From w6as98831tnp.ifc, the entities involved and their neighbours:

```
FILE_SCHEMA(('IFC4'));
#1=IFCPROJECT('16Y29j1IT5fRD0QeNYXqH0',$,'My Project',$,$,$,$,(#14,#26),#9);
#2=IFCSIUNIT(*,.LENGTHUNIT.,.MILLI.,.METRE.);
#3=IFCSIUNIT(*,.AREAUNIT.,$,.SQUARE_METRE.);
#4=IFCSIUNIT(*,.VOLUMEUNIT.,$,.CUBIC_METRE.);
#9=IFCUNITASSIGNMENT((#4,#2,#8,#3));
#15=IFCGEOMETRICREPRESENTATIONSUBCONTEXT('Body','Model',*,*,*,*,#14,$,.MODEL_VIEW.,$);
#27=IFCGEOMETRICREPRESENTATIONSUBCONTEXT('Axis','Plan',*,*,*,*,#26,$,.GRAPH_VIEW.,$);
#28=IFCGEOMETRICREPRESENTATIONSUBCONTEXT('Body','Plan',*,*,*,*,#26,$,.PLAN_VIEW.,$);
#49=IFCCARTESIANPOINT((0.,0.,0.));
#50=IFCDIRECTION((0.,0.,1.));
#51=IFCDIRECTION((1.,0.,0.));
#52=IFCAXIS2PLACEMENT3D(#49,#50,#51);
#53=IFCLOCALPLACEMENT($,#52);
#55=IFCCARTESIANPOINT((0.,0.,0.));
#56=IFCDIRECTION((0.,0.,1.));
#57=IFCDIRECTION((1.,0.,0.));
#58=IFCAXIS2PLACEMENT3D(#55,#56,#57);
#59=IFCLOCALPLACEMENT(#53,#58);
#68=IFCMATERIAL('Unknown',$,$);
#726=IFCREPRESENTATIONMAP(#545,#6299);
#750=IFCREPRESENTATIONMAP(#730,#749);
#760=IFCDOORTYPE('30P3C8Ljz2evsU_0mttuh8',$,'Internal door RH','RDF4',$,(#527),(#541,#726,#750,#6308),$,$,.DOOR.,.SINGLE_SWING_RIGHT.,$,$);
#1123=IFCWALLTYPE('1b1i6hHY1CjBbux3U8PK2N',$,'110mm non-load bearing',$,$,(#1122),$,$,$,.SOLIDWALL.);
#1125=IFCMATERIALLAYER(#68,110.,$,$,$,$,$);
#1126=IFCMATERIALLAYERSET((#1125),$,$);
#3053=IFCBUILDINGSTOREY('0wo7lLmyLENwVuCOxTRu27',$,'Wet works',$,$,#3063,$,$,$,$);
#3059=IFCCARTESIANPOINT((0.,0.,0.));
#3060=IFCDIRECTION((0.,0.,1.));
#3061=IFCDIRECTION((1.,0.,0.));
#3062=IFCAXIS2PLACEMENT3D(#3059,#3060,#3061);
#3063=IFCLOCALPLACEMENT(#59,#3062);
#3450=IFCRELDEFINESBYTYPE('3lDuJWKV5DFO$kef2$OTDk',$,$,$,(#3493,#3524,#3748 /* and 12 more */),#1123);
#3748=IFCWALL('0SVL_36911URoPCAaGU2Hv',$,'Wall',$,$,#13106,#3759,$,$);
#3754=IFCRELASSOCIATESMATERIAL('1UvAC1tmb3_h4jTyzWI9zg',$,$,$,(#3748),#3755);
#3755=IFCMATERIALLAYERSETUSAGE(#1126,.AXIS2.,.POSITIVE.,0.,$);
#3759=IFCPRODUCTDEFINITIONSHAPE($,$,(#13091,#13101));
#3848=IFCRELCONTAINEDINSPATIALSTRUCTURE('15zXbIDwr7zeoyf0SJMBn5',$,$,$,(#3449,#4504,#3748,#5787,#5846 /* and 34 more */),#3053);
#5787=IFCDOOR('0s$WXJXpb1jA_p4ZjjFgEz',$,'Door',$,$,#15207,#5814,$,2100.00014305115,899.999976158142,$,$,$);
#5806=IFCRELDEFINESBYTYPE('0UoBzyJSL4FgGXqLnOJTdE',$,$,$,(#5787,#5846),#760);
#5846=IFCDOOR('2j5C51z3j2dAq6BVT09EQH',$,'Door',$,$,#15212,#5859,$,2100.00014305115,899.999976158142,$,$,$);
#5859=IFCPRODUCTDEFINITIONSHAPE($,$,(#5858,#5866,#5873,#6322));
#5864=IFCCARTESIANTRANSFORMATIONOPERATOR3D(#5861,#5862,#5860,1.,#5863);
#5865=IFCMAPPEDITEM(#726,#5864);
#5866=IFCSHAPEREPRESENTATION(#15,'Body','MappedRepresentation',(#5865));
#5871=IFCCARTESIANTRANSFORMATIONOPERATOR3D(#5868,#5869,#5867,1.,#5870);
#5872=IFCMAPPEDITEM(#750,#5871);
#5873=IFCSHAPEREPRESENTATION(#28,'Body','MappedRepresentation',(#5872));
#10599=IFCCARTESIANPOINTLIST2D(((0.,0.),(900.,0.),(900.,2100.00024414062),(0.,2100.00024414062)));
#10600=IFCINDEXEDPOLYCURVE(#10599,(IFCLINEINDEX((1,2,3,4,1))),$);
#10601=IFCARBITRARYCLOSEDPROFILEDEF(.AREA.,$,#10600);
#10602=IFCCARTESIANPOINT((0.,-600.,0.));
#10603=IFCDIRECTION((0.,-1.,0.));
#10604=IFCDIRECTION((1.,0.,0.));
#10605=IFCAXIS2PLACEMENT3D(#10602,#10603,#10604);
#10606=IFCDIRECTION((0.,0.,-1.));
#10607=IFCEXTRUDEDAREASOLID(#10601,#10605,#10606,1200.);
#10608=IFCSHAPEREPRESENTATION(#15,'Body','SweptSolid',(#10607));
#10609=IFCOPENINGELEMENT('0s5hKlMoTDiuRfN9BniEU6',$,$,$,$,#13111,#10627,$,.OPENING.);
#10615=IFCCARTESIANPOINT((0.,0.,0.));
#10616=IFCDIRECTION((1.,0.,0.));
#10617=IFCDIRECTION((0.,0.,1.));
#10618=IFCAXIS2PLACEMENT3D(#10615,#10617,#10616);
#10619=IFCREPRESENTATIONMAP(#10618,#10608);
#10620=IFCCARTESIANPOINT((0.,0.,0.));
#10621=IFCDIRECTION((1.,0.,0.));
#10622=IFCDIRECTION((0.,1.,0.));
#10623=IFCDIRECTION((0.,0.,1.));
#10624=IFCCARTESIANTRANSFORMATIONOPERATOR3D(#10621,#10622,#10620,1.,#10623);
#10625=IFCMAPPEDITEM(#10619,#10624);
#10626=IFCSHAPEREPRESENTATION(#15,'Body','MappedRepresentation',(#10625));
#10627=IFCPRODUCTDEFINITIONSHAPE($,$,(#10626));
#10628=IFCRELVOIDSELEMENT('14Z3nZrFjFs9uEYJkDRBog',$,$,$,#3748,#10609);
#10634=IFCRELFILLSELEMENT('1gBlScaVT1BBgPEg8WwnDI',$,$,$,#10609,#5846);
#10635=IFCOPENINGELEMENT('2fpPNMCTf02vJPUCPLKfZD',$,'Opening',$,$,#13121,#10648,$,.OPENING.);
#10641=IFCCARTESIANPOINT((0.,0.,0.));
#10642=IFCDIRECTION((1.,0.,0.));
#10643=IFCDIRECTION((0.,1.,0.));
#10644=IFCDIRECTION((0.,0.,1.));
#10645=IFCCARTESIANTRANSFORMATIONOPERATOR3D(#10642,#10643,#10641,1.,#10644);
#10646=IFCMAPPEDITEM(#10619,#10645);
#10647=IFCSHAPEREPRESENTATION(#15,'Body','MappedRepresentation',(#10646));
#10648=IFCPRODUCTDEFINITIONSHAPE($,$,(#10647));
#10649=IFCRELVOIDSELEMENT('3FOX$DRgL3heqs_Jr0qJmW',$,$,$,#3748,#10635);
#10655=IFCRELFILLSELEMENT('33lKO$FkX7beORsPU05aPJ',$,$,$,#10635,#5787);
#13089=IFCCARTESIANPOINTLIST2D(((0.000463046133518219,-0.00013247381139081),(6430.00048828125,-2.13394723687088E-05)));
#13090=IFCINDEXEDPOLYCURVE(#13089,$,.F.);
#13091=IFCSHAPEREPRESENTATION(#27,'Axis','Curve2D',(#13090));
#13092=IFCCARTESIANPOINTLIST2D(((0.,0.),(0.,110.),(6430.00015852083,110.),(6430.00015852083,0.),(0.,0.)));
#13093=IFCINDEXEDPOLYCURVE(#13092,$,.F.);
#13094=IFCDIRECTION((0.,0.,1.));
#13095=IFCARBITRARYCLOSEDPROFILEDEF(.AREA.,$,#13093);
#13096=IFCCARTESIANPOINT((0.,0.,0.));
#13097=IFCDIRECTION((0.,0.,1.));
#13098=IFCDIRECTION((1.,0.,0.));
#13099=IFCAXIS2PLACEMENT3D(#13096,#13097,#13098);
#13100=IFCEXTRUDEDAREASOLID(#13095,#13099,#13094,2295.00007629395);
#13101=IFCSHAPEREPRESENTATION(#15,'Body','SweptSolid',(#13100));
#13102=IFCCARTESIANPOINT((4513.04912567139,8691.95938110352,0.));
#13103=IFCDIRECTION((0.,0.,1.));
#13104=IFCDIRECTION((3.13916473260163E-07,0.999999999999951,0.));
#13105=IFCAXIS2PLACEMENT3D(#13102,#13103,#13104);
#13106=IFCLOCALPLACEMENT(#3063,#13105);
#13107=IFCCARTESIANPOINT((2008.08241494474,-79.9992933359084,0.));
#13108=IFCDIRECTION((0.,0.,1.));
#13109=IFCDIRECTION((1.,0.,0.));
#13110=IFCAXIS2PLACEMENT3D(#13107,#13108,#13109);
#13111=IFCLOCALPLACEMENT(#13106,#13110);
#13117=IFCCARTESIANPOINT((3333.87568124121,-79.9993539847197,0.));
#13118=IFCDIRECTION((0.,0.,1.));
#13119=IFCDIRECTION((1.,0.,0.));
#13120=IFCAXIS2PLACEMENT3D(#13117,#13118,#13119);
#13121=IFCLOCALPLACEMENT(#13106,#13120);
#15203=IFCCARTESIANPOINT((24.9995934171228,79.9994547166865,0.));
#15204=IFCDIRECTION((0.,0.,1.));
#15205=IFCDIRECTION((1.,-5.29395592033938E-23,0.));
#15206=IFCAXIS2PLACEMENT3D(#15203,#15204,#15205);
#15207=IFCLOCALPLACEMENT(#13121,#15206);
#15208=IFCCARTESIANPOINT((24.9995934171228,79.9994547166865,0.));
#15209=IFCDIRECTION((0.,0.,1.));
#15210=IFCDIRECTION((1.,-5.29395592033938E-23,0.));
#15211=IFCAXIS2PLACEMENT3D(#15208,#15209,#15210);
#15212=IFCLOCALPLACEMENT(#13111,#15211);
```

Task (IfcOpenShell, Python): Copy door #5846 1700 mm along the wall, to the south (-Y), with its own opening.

```python
import ifcopenshell
import ifcopenshell.api.feature
import ifcopenshell.api.geometry
import ifcopenshell.api.root
import ifcopenshell.geom
import ifcopenshell.util.element
import ifcopenshell.util.placement
import ifcopenshell.util.shape

model = ifcopenshell.open("w6as98831tnp.ifc")
settings = ifcopenshell.geom.settings()


def volume(element):
    """Net volume in cubic metres, openings subtracted."""
    shape = ifcopenshell.geom.create_shape(settings, element)
    return ifcopenshell.util.shape.get_volume(shape.geometry)


door = model.by_id(5846)
opening = door.FillsVoids[0].RelatingOpeningElement
wall = opening.VoidsElements[0].RelatingBuildingElement
before = volume(wall)
shift = ifcopenshell.util.placement.get_local_placement(wall.ObjectPlacement)[:3, 0] * -1700.0

# copy_class copies the void relationship, type, container and properties, but no geometry.
new_opening = ifcopenshell.api.root.copy_class(model, product=opening)
new_opening.Representation = ifcopenshell.util.element.copy_deep(
    model, opening.Representation, exclude=["IfcGeometricRepresentationContext", "IfcRepresentationMap"]
)
new_door = ifcopenshell.api.root.copy_class(model, product=door)
new_door.Representation = ifcopenshell.util.element.copy_deep(
    model, door.Representation, exclude=["IfcGeometricRepresentationContext", "IfcRepresentationMap"]
)
ifcopenshell.api.feature.add_filling(model, opening=new_opening, element=new_door)

for old, new in ((opening, new_opening), (door, new_door)):
    matrix = ifcopenshell.util.placement.get_local_placement(old.ObjectPlacement)
    matrix[:3, 3] += shift
    ifcopenshell.api.geometry.edit_object_placement(model, product=new, matrix=matrix, is_si=False)

after = volume(wall)

print(f"wall volume {before:.3f} -> {after:.3f} m3")

model.write("w6as98831tnp_updated.ifc")
```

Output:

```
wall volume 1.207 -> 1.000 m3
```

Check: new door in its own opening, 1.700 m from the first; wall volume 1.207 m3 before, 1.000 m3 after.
